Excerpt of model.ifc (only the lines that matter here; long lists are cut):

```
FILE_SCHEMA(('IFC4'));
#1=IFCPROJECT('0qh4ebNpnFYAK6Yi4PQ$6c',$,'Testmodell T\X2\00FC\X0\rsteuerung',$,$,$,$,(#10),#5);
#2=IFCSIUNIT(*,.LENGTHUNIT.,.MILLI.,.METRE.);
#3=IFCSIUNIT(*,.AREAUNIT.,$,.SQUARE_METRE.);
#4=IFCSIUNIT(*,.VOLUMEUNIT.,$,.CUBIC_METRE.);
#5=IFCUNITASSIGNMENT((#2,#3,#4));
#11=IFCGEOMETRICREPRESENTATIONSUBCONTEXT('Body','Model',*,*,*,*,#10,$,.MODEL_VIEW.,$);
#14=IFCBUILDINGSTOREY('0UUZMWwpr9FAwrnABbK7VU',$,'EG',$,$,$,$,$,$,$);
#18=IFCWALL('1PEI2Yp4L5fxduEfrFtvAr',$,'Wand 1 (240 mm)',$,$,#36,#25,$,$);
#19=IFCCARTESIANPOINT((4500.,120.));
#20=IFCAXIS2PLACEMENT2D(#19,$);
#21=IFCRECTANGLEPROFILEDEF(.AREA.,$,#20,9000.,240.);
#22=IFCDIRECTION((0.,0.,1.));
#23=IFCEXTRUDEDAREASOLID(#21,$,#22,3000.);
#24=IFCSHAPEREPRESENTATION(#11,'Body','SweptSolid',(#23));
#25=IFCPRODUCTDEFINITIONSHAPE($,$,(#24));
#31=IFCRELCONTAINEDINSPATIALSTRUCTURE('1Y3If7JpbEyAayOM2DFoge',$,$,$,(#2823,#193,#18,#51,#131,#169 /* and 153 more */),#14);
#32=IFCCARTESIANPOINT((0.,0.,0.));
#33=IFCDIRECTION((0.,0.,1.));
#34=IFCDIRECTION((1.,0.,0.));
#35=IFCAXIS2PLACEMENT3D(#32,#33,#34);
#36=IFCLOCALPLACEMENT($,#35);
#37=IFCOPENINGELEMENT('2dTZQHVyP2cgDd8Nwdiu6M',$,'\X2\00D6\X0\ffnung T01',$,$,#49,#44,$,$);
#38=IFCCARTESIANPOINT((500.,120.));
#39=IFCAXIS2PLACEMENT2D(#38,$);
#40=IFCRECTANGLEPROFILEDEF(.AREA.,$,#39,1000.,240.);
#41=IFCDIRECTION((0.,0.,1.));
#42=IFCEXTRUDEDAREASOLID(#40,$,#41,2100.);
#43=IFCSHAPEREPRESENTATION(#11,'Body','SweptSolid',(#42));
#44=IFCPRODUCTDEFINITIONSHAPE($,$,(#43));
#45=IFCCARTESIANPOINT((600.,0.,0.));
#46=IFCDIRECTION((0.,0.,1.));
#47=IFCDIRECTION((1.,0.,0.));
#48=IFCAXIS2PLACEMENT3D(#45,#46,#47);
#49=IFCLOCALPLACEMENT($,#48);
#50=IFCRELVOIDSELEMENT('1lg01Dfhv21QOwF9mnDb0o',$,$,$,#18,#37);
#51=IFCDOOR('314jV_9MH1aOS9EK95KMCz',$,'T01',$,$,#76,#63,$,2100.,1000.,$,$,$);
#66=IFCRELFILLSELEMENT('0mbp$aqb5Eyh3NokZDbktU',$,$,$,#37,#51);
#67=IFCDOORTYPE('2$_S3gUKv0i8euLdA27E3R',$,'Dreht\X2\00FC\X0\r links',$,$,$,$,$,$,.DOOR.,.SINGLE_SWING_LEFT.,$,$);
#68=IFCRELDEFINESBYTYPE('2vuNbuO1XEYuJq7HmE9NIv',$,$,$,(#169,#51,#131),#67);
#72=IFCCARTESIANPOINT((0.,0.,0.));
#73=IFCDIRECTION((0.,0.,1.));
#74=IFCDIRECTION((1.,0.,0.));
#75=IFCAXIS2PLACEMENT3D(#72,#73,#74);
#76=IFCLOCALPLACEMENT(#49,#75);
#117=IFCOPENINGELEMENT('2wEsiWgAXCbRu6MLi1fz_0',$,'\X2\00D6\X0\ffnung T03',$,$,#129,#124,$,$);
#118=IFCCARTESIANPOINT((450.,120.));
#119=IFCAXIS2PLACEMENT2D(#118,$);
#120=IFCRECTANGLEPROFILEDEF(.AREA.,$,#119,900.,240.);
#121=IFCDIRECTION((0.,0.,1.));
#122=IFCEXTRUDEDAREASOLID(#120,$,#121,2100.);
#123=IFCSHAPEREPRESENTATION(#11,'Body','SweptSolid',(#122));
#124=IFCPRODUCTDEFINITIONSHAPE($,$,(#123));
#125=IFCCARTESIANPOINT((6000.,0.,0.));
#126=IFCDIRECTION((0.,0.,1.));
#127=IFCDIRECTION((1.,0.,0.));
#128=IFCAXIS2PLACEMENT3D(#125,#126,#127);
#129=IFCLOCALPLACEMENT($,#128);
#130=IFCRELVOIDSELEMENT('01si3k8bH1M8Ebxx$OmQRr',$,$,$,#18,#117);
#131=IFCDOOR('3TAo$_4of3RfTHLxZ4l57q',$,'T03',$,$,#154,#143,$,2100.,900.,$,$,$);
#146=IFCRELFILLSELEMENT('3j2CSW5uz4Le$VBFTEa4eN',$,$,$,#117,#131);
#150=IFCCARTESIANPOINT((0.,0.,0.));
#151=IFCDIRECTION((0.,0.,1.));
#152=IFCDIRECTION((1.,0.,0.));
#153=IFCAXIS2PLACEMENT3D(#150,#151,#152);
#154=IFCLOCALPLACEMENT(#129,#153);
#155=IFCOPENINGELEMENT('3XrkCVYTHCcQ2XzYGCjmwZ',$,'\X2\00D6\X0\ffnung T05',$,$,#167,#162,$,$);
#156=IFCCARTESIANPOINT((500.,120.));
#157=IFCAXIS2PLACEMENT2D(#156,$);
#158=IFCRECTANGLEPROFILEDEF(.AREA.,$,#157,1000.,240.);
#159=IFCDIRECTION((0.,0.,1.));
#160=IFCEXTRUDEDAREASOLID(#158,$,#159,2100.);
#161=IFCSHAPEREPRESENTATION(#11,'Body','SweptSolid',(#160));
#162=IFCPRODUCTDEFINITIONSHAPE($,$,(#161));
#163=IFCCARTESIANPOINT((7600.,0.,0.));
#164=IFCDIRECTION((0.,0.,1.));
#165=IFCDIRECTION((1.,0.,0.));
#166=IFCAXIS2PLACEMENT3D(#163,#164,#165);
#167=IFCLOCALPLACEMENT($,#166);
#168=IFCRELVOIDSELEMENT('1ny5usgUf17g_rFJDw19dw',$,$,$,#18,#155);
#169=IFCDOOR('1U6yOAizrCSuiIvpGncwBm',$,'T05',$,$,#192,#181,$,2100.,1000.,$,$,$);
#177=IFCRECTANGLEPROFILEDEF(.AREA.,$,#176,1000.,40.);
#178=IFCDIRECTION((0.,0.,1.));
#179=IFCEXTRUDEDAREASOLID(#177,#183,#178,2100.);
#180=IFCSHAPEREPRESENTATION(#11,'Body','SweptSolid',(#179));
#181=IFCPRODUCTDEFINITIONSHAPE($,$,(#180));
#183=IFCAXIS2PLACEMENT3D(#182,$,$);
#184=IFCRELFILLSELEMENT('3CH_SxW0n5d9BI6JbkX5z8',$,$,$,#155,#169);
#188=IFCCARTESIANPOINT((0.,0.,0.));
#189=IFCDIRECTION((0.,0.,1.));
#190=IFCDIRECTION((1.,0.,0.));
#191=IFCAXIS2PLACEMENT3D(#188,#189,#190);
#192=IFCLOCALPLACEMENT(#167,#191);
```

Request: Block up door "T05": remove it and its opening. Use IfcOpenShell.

```python
import ifcopenshell
import ifcopenshell.api.feature
import ifcopenshell.api.root
import ifcopenshell.geom
import ifcopenshell.util.shape

model = ifcopenshell.open("model.ifc")
settings = ifcopenshell.geom.settings()


def volume(element):
    """Net volume in cubic metres, openings subtracted."""
    shape = ifcopenshell.geom.create_shape(settings, element)
    return ifcopenshell.util.shape.get_volume(shape.geometry)


door = model.by_guid("1U6yOAizrCSuiIvpGncwBm")
opening = door.FillsVoids[0].RelatingOpeningElement
wall = opening.VoidsElements[0].RelatingBuildingElement
before = volume(wall)

ifcopenshell.api.root.remove_product(model, product=door)
ifcopenshell.api.feature.remove_feature(model, feature=opening)

after = volume(wall)

print(f"wall volume {before:.3f} -> {after:.3f} m3")

model.write("model_updated.ifc")
```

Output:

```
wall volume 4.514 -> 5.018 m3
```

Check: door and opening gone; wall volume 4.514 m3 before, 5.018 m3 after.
